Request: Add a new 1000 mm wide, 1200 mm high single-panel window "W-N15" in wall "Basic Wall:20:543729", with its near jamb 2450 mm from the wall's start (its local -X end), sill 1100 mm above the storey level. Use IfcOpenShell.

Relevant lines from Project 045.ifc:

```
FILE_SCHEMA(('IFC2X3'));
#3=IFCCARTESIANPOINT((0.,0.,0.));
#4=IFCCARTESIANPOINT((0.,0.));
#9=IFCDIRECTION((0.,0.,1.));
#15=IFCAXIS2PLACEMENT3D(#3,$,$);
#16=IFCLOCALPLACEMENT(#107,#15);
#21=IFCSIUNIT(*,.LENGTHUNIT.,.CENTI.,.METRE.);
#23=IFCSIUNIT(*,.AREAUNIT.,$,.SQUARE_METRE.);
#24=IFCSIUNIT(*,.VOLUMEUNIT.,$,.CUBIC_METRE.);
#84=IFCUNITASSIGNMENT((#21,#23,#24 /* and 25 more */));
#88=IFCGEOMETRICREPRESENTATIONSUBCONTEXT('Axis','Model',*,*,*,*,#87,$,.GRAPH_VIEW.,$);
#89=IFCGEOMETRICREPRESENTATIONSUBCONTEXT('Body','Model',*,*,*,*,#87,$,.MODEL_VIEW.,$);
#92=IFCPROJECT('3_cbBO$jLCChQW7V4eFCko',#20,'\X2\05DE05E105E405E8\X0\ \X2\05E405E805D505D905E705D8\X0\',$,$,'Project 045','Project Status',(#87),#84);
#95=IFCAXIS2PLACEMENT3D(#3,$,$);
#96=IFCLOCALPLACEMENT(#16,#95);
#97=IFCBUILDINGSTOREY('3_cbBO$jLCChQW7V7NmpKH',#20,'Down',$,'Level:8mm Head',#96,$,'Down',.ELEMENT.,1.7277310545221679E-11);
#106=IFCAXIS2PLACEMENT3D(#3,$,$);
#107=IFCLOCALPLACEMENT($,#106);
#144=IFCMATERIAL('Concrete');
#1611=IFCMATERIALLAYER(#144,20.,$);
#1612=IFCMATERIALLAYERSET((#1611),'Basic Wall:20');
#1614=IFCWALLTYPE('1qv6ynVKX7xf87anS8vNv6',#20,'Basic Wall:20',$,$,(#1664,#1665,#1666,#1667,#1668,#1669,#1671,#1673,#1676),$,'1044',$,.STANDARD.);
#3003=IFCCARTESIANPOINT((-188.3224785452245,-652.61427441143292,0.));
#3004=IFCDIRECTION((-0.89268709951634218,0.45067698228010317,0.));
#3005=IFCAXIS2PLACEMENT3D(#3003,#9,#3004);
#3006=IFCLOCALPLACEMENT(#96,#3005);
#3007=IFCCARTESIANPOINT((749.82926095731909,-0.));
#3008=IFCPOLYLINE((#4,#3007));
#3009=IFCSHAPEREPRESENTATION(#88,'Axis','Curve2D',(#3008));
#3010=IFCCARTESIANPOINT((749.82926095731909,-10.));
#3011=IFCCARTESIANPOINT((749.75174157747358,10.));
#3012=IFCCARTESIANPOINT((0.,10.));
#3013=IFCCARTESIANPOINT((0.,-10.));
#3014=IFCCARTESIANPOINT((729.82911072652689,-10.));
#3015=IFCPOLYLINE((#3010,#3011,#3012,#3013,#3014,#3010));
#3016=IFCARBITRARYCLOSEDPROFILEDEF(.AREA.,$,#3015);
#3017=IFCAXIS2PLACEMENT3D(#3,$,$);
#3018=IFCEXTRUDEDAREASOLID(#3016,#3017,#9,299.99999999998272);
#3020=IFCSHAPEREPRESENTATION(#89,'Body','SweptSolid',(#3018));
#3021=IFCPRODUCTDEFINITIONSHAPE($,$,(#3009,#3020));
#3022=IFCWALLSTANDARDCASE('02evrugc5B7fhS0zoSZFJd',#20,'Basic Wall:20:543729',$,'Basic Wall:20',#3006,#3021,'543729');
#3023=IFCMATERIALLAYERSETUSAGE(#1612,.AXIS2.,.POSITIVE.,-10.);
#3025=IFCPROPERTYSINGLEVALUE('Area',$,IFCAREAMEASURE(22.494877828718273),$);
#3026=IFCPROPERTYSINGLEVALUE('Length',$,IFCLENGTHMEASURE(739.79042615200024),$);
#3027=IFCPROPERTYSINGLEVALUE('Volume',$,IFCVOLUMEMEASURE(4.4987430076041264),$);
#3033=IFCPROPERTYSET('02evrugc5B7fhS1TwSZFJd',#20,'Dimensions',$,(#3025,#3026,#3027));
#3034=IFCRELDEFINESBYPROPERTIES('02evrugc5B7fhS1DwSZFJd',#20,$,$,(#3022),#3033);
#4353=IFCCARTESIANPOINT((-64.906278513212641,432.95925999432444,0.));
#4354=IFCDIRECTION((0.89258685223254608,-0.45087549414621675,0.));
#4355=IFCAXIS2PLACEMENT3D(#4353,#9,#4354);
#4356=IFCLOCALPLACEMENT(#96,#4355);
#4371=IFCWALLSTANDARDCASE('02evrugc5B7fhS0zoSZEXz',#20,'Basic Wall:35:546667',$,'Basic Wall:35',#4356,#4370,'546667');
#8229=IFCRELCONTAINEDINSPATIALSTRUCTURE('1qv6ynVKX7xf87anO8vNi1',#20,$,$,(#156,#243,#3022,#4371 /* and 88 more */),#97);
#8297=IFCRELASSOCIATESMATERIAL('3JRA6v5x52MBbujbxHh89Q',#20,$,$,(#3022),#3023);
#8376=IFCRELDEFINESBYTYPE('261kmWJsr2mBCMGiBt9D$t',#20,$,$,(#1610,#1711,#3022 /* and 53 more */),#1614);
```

```python
import numpy as np
import ifcopenshell
import ifcopenshell.api.feature
import ifcopenshell.api.geometry
import ifcopenshell.api.pset
import ifcopenshell.api.root
import ifcopenshell.api.spatial
import ifcopenshell.api.type
import ifcopenshell.geom
import ifcopenshell.util.element
import ifcopenshell.util.placement
import ifcopenshell.util.representation
import ifcopenshell.util.shape
import ifcopenshell.util.unit

model = ifcopenshell.open("Project 045.ifc")
unit_scale = ifcopenshell.util.unit.calculate_unit_scale(model)
area_scale = ifcopenshell.util.unit.calculate_unit_scale(model, "AREAUNIT")
volume_scale = ifcopenshell.util.unit.calculate_unit_scale(model, "VOLUMEUNIT")
settings = ifcopenshell.geom.settings()


def volume(element):
    """Net volume in cubic metres, openings subtracted."""
    shape = ifcopenshell.geom.create_shape(settings, element)
    return ifcopenshell.util.shape.get_volume(shape.geometry)


wall = model.by_guid("02evrugc5B7fhS0zoSZFJd")
storey = ifcopenshell.util.element.get_container(wall, ifc_class="IfcBuildingStorey")
context = ifcopenshell.util.representation.get_context(model, "Model", "Body", "MODEL_VIEW")
before = volume(wall)

width, height, from_end, sill = 1, 1.2, 2.45, 1.1  # metres

# The wall runs along its own X axis, and the end named is its -X end.
wall_shape = ifcopenshell.geom.create_shape(settings, wall)
x, y, z = ifcopenshell.util.shape.get_vertices(wall_shape.geometry).T
start = x.min() + from_end
face, thickness = float(y.min()), float(y.max() - y.min())
wall_matrix = ifcopenshell.util.placement.get_local_placement(wall.ObjectPlacement)
level = ifcopenshell.util.placement.get_local_placement(storey.ObjectPlacement)[2, 3]


def in_wall(x, y):
    """Placement at x, y metres in the wall's axes, at sill height."""
    matrix = wall_matrix.copy()
    matrix[:, 3] = wall_matrix @ np.array([x / unit_scale, y / unit_scale, 0.0, 1.0])
    matrix[2, 3] = level + sill / unit_scale
    return matrix


# Opening: a box that overshoots both wall faces by 50 mm.
opening = ifcopenshell.api.root.create_entity(model, ifc_class="IfcOpeningElement")
box = ifcopenshell.api.geometry.add_wall_representation(
    model, context=context, length=width, height=height, thickness=thickness + 0.1
)
ifcopenshell.api.geometry.assign_representation(model, product=opening, representation=box)
ifcopenshell.api.geometry.edit_object_placement(model, product=opening, matrix=in_wall(start, face - 0.05), is_si=False)
ifcopenshell.api.feature.add_feature(model, feature=opening, element=wall)

window = ifcopenshell.api.root.create_entity(model, ifc_class="IfcWindow", name="W-N15")
window.OverallWidth, window.OverallHeight = width / unit_scale, height / unit_scale
body = ifcopenshell.api.geometry.add_window_representation(
    model,
    context=context,
    overall_width=window.OverallWidth,
    overall_height=window.OverallHeight,
    partition_type="SINGLE_PANEL",
)
ifcopenshell.api.geometry.assign_representation(model, product=window, representation=body)
ifcopenshell.api.spatial.assign_container(model, products=[window], relating_structure=storey)
fills = ifcopenshell.api.feature.add_filling(model, opening=opening, element=window)
fills.OwnerHistory = window.OwnerHistory  # required in IFC2X3

# IFC2X3 keeps the operation on the window style.
style = ifcopenshell.api.root.create_entity(model, ifc_class="IfcWindowStyle", name="W-N15")
style.OperationType, style.ConstructionType = "SINGLE_PANEL", "NOTDEFINED"
style.ParameterTakesPrecedence = style.Sizeable = False
ifcopenshell.api.type.assign_type(model, related_objects=[window], relating_type=style)

# Centre the window in the wall's thickness.
ifcopenshell.api.geometry.edit_object_placement(model, product=window, matrix=in_wall(start, face), is_si=False)
window_shape = ifcopenshell.geom.create_shape(settings, window)
depth = ifcopenshell.util.shape.get_vertices(window_shape.geometry)[:, 1]
offset = face + thickness / 2 - (depth.min() + depth.max()) / 2
ifcopenshell.api.geometry.edit_object_placement(model, product=window, matrix=in_wall(start, offset), is_si=False)

after = volume(wall)

# Update the wall's stored quantities.
pset = model.by_id(ifcopenshell.util.element.get_pset(wall, "Dimensions", should_inherit=False)["id"])
ifcopenshell.api.pset.edit_pset(model, pset=pset, properties={
    "Area": model.create_entity("IfcAreaMeasure", after / thickness / area_scale),
    "Volume": model.create_entity("IfcVolumeMeasure", after / volume_scale),
})

print(f"wall volume {before:.3f} -> {after:.3f} m3")

model.write("Project 045_edited.ifc")
```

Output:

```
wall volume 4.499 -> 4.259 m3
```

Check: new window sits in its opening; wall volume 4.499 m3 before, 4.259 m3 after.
